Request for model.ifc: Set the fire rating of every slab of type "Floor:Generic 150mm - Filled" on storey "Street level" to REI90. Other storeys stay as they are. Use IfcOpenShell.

First a look at what the model holds.

```python
import ifcopenshell
import ifcopenshell.util.element

model = ifcopenshell.open("model.ifc")
print(model.schema)
storey = next(s for s in model.by_type("IfcBuildingStorey") if s.Name == "Street level")
slabs = [e for e in ifcopenshell.util.element.get_decomposition(storey) if e.is_a("IfcSlab")]
seen = {}
for e in slabs:
    element_type = ifcopenshell.util.element.get_type(e)
    key = (element_type.Name if element_type != e and element_type else None, ifcopenshell.util.element.get_pset(e, "Pset_SlabCommon", "FireRating"))
    seen[key] = seen.get(key, 0) + 1
for (name, value), count in sorted(seen.items(), key=str):
    print(count, "x", name, "|", value)
```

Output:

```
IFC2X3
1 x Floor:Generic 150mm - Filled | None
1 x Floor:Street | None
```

```python
import ifcopenshell
import ifcopenshell.api.pset
import ifcopenshell.util.element

model = ifcopenshell.open("model.ifc")

storey = next(s for s in model.by_type("IfcBuildingStorey") if s.Name == "Street level")
slabs = [e for e in ifcopenshell.util.element.get_decomposition(storey) if e.is_a("IfcSlab")]

count = 0
for e in slabs:
    element_type = ifcopenshell.util.element.get_type(e)
    if element_type in (None, e) or element_type.Name != "Floor:Generic 150mm - Filled":
        continue
    # add_pset returns the element's existing set when there is one.
    pset = ifcopenshell.api.pset.add_pset(model, product=e, name="Pset_SlabCommon")
    ifcopenshell.api.pset.edit_pset(model, pset=pset, properties={"FireRating": "REI90"})
    count += 1

print(count, "slabs updated")

model.write("model_updated.ifc")
```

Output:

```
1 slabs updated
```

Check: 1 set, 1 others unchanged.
